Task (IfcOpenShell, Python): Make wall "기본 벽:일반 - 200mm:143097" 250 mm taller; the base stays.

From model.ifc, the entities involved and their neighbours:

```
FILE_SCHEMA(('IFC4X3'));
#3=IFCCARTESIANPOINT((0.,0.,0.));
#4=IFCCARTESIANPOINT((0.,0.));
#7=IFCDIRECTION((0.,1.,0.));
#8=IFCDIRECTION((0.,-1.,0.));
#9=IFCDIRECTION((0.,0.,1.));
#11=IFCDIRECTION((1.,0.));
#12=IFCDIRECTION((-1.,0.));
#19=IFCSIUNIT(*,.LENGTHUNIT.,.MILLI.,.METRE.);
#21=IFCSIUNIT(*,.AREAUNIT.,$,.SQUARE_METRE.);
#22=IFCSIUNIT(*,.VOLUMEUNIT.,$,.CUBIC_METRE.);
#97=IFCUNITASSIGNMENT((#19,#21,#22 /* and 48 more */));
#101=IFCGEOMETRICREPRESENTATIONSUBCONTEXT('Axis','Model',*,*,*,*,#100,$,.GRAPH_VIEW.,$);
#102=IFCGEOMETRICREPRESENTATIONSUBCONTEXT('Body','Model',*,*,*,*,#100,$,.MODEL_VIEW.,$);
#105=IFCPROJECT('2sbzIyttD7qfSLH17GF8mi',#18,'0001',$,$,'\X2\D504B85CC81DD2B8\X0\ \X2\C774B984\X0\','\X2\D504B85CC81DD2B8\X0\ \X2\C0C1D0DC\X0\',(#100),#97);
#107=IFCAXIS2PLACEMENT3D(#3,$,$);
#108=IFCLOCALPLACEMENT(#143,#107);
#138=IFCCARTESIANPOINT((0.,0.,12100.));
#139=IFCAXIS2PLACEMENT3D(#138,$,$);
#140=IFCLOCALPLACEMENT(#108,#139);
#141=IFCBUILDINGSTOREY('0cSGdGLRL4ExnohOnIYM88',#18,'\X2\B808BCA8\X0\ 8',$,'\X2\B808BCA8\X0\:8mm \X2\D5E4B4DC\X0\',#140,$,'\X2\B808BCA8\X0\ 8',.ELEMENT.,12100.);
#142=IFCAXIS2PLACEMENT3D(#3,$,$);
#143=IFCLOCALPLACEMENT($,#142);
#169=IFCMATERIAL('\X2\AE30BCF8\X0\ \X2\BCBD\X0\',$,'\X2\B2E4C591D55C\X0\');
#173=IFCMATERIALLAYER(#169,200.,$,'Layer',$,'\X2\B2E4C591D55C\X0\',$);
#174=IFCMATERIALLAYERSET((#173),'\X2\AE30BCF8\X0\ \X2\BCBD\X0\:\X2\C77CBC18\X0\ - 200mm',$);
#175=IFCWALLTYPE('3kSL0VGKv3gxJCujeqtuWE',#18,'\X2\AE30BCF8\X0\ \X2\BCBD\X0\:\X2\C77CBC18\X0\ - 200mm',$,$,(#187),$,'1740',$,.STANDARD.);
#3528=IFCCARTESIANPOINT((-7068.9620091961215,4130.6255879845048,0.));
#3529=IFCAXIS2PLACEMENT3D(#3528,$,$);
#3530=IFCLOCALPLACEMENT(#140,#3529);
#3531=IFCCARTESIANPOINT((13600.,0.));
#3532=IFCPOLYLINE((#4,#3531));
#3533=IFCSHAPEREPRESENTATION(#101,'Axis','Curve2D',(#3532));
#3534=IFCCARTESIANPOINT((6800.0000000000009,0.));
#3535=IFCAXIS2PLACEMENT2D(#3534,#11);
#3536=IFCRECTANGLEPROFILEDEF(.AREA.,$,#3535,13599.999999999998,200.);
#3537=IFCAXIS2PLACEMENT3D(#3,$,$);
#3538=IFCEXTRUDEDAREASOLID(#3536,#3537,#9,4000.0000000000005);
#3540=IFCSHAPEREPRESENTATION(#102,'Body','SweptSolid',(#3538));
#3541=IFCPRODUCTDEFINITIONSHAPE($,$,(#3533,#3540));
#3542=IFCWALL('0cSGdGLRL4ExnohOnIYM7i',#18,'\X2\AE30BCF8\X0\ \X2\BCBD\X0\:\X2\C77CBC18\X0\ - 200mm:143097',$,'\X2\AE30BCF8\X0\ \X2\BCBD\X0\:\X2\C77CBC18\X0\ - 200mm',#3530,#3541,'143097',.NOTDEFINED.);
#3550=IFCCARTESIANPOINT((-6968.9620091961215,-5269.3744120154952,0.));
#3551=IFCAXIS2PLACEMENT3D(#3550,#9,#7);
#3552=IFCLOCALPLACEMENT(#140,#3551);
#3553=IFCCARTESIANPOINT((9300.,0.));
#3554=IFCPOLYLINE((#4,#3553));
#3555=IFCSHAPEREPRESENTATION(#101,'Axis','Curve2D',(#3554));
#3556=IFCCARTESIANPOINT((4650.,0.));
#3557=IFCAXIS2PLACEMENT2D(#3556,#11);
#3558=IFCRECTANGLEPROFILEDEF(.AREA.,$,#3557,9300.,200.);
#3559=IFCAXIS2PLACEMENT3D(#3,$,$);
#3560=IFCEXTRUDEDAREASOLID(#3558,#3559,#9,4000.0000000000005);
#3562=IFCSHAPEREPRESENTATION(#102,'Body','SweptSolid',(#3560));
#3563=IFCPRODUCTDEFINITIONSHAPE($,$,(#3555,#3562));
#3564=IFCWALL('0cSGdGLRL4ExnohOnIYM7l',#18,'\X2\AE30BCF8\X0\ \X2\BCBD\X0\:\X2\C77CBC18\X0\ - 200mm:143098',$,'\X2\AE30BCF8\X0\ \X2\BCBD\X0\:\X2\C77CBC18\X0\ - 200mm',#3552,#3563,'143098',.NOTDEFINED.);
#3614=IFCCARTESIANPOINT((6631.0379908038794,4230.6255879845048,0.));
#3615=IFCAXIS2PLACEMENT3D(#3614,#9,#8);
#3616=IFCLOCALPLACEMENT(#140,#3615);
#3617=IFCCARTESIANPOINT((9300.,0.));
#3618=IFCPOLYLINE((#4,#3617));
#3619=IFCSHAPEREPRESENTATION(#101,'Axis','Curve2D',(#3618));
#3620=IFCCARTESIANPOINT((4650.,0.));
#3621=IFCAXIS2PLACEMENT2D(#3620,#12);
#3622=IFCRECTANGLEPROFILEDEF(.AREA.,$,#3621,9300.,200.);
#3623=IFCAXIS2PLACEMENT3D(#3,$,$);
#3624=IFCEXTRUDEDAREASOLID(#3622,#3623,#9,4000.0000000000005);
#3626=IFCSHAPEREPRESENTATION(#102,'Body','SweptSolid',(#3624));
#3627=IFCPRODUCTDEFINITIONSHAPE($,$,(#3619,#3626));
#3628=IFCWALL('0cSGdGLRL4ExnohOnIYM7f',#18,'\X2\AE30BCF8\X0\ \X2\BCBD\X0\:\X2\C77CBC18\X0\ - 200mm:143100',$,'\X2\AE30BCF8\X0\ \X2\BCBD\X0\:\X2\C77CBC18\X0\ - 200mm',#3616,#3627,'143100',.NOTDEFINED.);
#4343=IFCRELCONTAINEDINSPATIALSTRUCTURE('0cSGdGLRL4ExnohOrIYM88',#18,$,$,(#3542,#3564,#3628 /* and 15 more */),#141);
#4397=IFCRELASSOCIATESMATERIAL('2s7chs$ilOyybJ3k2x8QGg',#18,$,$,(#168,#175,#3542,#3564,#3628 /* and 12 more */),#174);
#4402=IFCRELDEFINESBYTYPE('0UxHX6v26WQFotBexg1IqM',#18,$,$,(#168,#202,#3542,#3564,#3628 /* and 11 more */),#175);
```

```python
import ifcopenshell
import ifcopenshell.geom
import ifcopenshell.util.representation
import ifcopenshell.util.shape
import ifcopenshell.util.unit

model = ifcopenshell.open("model.ifc")
unit_scale = ifcopenshell.util.unit.calculate_unit_scale(model)
settings = ifcopenshell.geom.settings()


def volume(element):
    """Net volume in cubic metres, openings subtracted."""
    shape = ifcopenshell.geom.create_shape(settings, element)
    return ifcopenshell.util.shape.get_volume(shape.geometry)


wall = model.by_guid("0cSGdGLRL4ExnohOnIYM7i")
before = volume(wall)

body = ifcopenshell.util.representation.get_representation(wall, "Model", "Body")
solid = body.Items[0]
old_height = solid.Depth
solid.Depth += 0.25 / unit_scale
after = volume(wall)

print(f"height {old_height:g} -> {solid.Depth:g}, volume {before:.3f} -> {after:.3f} m3")

model.write("model_edited.ifc")
```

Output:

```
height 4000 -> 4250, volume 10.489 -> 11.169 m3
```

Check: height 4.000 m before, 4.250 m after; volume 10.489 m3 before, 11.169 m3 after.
